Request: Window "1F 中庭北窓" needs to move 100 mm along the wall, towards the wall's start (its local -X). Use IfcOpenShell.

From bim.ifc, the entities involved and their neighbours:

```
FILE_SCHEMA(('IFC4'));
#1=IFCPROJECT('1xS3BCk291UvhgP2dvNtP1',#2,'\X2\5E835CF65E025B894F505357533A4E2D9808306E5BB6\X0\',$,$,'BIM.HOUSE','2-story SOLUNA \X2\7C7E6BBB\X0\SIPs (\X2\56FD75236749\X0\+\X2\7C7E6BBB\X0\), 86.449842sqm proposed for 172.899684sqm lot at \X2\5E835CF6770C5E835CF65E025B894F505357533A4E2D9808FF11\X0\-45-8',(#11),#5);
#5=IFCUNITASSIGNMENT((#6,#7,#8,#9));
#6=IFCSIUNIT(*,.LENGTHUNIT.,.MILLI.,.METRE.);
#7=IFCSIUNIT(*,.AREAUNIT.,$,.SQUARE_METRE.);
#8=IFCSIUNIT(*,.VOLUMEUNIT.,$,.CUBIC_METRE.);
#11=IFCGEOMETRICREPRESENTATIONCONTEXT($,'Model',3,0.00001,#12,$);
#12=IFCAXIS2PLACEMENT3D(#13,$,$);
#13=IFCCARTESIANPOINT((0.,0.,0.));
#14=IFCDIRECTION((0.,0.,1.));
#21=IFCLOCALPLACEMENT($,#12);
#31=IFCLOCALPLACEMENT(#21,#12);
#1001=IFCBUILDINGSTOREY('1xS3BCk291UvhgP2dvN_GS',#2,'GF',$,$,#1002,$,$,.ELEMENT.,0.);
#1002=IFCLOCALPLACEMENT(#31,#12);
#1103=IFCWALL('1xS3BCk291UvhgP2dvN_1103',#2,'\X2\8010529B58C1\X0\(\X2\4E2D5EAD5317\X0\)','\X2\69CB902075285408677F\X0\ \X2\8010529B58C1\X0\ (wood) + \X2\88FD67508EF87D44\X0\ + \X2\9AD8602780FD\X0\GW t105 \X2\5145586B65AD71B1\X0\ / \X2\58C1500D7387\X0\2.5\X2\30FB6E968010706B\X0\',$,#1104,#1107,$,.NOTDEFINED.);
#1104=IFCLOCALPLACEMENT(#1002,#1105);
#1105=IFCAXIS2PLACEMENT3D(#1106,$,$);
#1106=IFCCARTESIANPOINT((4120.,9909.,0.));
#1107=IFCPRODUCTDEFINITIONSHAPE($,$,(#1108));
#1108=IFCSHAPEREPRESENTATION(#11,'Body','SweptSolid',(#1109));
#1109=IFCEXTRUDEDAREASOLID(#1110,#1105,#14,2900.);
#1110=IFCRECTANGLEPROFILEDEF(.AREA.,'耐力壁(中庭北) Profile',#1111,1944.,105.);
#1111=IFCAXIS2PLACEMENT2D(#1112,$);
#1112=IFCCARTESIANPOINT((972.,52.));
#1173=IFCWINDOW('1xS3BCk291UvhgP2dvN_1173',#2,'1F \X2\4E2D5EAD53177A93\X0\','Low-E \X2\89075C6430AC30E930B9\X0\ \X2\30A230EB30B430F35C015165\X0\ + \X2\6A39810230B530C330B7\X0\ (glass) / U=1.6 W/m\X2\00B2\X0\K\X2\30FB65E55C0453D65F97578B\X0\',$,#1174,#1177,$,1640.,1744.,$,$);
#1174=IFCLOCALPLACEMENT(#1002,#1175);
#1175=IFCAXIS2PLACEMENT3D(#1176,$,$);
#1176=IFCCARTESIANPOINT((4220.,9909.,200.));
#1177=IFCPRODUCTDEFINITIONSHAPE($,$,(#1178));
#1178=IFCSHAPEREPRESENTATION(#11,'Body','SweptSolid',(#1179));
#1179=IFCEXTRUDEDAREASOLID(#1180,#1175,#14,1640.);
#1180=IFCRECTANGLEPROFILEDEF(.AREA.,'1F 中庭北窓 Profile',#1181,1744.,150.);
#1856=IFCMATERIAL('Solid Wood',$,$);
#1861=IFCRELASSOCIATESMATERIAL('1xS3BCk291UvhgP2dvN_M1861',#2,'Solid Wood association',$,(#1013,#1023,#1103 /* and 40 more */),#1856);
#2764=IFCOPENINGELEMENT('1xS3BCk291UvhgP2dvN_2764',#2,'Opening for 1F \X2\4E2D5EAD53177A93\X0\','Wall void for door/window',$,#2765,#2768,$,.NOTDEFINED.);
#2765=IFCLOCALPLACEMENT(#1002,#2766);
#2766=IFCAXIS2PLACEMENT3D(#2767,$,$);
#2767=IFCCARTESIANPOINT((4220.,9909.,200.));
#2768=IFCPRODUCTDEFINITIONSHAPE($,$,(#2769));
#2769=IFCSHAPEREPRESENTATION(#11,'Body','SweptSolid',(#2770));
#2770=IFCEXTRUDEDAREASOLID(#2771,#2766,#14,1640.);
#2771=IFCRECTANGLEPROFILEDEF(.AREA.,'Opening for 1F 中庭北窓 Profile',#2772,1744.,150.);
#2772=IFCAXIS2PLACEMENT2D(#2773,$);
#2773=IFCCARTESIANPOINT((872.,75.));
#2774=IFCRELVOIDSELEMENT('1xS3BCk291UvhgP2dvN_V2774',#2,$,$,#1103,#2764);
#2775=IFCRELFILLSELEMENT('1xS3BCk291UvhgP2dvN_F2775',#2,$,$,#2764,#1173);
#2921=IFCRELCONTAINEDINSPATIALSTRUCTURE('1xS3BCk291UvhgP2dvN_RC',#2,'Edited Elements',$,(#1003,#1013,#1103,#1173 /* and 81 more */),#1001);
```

```python
import ifcopenshell
import ifcopenshell.api.geometry
import ifcopenshell.util.placement
import ifcopenshell.util.unit

model = ifcopenshell.open("bim.ifc")
unit_scale = ifcopenshell.util.unit.calculate_unit_scale(model)

window = model.by_guid("1xS3BCk291UvhgP2dvN_1173")
opening = window.FillsVoids[0].RelatingOpeningElement
wall = opening.VoidsElements[0].RelatingBuildingElement

wall_matrix = ifcopenshell.util.placement.get_local_placement(wall.ObjectPlacement)
shift = wall_matrix[:3, 0] * -0.1 / unit_scale
before = ifcopenshell.util.placement.get_local_placement(window.ObjectPlacement)[:3, 3].copy()

# The window is not placed relative to its opening, so move both.
for product in (opening, window):
    matrix = ifcopenshell.util.placement.get_local_placement(product.ObjectPlacement)
    matrix[:3, 3] += shift
    ifcopenshell.api.geometry.edit_object_placement(model, product=product, matrix=matrix, is_si=False)

after = ifcopenshell.util.placement.get_local_placement(window.ObjectPlacement)[:3, 3]
print("window moved by", (after - before).round(3) + 0.0)

model.write("bim_updated.ifc")
```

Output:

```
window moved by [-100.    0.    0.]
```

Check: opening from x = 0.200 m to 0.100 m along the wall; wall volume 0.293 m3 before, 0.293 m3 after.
